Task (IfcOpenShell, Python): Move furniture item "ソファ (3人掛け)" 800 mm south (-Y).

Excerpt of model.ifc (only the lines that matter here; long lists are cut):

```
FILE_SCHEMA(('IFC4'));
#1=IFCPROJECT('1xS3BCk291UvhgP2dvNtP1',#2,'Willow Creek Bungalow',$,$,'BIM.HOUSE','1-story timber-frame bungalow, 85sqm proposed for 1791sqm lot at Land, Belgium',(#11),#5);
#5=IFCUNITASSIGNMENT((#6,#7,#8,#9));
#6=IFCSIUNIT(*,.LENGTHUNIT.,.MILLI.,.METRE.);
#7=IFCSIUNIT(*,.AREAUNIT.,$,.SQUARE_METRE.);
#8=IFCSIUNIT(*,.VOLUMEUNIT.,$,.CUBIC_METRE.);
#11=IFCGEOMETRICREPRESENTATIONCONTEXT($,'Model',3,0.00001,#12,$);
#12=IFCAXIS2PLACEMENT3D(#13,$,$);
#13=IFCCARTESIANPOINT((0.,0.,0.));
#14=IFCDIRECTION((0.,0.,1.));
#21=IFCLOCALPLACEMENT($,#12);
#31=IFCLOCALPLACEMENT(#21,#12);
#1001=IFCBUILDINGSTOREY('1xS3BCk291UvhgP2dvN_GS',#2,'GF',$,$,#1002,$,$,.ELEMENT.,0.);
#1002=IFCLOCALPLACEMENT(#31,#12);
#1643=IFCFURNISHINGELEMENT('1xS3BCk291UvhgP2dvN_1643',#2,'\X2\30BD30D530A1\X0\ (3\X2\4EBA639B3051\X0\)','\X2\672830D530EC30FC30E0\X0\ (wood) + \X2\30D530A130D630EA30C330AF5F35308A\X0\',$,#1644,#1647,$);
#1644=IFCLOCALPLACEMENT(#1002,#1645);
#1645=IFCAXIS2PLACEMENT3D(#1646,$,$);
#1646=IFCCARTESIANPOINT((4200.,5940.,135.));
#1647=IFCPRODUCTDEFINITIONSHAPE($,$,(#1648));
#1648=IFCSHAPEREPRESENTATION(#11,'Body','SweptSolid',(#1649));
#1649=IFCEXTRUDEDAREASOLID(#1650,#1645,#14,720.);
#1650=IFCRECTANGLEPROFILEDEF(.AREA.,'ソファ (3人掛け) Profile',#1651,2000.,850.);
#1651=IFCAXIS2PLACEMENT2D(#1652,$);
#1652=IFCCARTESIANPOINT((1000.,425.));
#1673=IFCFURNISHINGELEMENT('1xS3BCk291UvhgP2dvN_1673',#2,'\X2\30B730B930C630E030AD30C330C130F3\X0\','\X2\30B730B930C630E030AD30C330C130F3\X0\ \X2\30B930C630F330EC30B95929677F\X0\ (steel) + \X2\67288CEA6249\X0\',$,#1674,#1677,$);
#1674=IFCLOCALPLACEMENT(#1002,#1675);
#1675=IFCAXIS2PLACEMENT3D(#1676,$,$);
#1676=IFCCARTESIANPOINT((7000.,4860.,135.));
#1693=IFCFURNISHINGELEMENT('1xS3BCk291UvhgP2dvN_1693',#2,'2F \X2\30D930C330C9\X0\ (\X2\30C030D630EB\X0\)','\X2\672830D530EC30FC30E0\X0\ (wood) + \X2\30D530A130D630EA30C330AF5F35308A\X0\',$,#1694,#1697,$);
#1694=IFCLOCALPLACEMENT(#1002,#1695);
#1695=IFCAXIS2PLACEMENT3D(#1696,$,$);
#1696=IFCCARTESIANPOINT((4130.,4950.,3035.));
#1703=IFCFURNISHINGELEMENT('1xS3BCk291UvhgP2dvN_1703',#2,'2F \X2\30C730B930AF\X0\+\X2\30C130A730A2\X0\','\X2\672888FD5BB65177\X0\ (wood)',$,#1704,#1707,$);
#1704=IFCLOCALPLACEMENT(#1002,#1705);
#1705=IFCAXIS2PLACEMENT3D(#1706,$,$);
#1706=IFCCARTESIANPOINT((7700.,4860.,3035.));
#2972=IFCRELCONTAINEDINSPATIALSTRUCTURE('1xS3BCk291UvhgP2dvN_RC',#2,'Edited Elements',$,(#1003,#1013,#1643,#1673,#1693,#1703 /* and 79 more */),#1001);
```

```python
import ifcopenshell
import ifcopenshell.api.geometry
import ifcopenshell.util.placement

model = ifcopenshell.open("model.ifc")

item = model.by_guid("1xS3BCk291UvhgP2dvN_1643")
matrix = ifcopenshell.util.placement.get_local_placement(item.ObjectPlacement)
matrix[1, 3] -= 800.0
ifcopenshell.api.geometry.edit_object_placement(model, product=item, matrix=matrix, is_si=False)

print(ifcopenshell.util.placement.get_local_placement(item.ObjectPlacement).round(3) + 0.0)

model.write("model_rev.ifc")
```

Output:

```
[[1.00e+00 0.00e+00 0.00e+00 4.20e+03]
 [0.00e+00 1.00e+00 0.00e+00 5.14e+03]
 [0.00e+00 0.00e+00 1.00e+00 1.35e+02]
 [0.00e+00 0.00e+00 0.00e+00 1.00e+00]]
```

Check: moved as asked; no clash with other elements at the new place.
